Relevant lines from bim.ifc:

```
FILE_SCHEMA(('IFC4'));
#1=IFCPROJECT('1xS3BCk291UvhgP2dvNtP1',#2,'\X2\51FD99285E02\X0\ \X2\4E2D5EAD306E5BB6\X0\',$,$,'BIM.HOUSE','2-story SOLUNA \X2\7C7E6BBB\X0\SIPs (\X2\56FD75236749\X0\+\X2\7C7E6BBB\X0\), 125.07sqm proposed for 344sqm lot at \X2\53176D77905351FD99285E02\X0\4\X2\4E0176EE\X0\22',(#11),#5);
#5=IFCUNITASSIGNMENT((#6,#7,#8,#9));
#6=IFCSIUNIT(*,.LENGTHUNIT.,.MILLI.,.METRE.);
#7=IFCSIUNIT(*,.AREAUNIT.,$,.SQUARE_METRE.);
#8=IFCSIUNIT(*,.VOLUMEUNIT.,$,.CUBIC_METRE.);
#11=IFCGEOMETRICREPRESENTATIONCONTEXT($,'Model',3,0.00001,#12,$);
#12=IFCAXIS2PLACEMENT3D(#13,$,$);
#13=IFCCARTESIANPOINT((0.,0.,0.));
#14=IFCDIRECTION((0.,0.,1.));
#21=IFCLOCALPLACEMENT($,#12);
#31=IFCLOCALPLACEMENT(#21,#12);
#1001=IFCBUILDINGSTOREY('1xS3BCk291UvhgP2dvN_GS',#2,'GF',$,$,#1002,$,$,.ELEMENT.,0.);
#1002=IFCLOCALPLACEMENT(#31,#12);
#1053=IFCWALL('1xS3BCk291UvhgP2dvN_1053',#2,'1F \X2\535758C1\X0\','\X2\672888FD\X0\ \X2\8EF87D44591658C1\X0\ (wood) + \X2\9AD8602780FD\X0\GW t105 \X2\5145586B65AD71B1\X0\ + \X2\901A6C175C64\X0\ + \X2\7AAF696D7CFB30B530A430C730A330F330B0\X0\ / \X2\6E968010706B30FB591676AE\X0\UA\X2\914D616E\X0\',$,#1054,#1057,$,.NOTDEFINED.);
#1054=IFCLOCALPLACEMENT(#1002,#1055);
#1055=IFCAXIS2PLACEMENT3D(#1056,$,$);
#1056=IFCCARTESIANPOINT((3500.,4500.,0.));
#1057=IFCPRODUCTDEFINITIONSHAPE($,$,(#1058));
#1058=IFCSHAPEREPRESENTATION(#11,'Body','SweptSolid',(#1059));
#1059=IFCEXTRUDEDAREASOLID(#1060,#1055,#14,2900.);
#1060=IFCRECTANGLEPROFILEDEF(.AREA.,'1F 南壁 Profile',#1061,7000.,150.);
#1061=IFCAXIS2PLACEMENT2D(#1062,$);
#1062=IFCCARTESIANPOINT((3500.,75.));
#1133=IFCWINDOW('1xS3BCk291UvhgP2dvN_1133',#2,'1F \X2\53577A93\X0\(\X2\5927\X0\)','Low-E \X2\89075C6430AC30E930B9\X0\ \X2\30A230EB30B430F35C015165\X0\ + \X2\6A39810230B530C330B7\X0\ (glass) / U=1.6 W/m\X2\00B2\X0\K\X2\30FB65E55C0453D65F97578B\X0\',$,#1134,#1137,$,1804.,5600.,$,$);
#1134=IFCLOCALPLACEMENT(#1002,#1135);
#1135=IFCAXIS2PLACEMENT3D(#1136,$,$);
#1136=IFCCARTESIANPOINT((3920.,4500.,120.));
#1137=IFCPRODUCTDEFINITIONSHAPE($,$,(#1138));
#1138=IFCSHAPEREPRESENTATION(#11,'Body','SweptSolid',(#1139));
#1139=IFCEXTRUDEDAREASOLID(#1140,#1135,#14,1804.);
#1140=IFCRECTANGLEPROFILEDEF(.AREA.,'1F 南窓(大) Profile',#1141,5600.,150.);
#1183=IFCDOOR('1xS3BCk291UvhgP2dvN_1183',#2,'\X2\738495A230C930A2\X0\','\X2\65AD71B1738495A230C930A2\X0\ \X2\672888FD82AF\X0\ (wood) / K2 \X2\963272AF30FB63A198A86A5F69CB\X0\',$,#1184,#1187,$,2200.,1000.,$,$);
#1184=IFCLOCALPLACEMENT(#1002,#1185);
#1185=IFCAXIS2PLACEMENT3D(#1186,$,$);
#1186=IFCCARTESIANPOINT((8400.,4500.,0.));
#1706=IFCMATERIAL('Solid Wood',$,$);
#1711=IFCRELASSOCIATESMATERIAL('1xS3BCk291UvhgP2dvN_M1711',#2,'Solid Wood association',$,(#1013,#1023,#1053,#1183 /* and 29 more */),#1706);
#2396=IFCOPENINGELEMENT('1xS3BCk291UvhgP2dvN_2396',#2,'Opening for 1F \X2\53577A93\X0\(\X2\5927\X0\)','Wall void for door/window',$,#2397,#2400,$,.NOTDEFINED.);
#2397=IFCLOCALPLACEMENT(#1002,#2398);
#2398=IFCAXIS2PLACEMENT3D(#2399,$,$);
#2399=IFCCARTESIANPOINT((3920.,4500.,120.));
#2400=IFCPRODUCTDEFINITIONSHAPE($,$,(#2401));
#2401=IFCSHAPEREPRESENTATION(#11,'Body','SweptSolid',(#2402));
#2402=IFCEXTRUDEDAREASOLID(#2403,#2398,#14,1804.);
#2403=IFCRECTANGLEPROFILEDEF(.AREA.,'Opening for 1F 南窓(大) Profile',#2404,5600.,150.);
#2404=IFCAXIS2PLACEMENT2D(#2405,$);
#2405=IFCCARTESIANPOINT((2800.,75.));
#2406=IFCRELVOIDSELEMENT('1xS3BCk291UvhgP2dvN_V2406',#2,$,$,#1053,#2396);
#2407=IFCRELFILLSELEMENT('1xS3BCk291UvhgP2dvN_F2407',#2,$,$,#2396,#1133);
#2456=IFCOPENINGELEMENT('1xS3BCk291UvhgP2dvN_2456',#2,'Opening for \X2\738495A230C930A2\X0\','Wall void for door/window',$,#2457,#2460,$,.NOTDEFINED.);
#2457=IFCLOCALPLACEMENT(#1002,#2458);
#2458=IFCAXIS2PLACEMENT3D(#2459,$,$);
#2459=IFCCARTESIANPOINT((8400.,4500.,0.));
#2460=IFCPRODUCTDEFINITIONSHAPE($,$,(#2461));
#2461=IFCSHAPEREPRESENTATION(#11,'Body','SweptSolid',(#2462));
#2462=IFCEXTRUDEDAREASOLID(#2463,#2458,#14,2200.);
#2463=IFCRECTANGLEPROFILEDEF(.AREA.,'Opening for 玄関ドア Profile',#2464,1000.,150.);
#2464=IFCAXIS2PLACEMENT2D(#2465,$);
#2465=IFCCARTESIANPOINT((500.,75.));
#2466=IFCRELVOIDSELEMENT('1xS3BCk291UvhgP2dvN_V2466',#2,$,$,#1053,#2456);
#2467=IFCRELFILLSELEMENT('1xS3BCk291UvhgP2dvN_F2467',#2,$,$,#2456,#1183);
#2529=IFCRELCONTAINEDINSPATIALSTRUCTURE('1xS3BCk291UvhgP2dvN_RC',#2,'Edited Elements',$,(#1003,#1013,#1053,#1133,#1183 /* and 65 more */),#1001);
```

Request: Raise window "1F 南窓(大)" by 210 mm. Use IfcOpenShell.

```python
import numpy as np
import ifcopenshell
import ifcopenshell.api.geometry
import ifcopenshell.util.placement
import ifcopenshell.util.unit

model = ifcopenshell.open("bim.ifc")
unit_scale = ifcopenshell.util.unit.calculate_unit_scale(model)

window = model.by_guid("1xS3BCk291UvhgP2dvN_1133")
opening = window.FillsVoids[0].RelatingOpeningElement
dz = 210.0

shift = np.array([0.0, 0.0, dz])
# The window is not placed relative to its opening, so move both.
for product in (opening, window):
    matrix = ifcopenshell.util.placement.get_local_placement(product.ObjectPlacement)
    matrix[:3, 3] += shift
    ifcopenshell.api.geometry.edit_object_placement(model, product=product, matrix=matrix, is_si=False)

print(f"moved by {dz * unit_scale:+.3f} m")

model.write("bim_v2.ifc")
```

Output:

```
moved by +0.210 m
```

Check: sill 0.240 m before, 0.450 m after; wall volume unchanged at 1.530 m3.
